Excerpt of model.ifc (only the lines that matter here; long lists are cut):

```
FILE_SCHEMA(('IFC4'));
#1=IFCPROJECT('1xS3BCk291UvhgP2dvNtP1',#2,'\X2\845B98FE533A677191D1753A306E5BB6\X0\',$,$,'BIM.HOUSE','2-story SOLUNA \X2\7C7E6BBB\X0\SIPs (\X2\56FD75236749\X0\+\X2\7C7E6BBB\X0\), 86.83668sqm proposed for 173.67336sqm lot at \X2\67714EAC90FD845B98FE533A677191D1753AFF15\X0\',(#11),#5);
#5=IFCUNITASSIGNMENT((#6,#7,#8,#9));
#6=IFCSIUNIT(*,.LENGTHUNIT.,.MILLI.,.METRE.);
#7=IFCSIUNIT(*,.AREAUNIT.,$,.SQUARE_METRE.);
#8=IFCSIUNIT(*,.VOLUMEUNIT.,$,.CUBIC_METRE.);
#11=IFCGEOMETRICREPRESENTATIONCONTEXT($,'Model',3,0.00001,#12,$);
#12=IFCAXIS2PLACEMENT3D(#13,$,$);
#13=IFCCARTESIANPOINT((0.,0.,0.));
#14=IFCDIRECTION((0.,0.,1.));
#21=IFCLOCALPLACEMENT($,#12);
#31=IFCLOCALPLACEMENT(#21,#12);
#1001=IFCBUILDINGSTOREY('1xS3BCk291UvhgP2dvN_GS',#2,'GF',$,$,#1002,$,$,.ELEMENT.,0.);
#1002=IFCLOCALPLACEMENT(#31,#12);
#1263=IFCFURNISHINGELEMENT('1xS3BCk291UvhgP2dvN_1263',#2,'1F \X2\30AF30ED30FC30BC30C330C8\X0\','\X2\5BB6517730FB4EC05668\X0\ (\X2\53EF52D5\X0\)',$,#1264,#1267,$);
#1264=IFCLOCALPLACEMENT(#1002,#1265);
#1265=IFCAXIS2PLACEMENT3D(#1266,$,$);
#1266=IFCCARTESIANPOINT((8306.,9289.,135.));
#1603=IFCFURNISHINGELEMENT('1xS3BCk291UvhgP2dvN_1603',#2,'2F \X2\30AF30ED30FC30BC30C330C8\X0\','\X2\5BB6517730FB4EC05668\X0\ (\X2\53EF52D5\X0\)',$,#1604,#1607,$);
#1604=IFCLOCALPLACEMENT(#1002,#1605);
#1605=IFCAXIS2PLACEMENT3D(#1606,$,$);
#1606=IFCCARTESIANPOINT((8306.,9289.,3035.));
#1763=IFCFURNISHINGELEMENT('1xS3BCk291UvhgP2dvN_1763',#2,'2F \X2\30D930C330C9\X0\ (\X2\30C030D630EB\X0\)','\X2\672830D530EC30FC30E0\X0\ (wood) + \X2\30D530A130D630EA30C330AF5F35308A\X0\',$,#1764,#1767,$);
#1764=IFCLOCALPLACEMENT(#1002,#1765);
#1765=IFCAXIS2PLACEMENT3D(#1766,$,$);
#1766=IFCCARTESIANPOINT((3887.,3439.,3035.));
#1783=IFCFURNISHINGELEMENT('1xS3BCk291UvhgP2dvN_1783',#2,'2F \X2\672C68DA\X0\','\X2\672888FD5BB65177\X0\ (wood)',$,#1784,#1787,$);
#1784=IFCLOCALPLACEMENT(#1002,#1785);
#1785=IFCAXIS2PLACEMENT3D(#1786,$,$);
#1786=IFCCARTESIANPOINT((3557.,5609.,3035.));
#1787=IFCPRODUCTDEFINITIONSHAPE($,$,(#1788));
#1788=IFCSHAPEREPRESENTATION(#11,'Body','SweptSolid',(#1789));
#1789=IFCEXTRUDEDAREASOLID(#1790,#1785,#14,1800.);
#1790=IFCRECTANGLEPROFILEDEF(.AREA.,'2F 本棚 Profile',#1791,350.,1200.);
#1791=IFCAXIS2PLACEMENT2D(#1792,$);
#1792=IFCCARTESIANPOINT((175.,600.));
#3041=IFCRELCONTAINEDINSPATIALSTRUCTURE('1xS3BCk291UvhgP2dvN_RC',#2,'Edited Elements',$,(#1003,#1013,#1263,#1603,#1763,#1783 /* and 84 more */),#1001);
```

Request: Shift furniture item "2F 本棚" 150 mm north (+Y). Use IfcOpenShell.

```python
import ifcopenshell
import ifcopenshell.api.geometry
import ifcopenshell.util.placement
import ifcopenshell.util.unit

model = ifcopenshell.open("model.ifc")
unit_scale = ifcopenshell.util.unit.calculate_unit_scale(model)

item = model.by_id(1783)
matrix = ifcopenshell.util.placement.get_local_placement(item.ObjectPlacement)
matrix[1, 3] += 0.15 / unit_scale
ifcopenshell.api.geometry.edit_object_placement(model, product=item, matrix=matrix, is_si=False)

print(ifcopenshell.util.placement.get_local_placement(item.ObjectPlacement).round(3) + 0.0)

model.write("model_updated.ifc")
```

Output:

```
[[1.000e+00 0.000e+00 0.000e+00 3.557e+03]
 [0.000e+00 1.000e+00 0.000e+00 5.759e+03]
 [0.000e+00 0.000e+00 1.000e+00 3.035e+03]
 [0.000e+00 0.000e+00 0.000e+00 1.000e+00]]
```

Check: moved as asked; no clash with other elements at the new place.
